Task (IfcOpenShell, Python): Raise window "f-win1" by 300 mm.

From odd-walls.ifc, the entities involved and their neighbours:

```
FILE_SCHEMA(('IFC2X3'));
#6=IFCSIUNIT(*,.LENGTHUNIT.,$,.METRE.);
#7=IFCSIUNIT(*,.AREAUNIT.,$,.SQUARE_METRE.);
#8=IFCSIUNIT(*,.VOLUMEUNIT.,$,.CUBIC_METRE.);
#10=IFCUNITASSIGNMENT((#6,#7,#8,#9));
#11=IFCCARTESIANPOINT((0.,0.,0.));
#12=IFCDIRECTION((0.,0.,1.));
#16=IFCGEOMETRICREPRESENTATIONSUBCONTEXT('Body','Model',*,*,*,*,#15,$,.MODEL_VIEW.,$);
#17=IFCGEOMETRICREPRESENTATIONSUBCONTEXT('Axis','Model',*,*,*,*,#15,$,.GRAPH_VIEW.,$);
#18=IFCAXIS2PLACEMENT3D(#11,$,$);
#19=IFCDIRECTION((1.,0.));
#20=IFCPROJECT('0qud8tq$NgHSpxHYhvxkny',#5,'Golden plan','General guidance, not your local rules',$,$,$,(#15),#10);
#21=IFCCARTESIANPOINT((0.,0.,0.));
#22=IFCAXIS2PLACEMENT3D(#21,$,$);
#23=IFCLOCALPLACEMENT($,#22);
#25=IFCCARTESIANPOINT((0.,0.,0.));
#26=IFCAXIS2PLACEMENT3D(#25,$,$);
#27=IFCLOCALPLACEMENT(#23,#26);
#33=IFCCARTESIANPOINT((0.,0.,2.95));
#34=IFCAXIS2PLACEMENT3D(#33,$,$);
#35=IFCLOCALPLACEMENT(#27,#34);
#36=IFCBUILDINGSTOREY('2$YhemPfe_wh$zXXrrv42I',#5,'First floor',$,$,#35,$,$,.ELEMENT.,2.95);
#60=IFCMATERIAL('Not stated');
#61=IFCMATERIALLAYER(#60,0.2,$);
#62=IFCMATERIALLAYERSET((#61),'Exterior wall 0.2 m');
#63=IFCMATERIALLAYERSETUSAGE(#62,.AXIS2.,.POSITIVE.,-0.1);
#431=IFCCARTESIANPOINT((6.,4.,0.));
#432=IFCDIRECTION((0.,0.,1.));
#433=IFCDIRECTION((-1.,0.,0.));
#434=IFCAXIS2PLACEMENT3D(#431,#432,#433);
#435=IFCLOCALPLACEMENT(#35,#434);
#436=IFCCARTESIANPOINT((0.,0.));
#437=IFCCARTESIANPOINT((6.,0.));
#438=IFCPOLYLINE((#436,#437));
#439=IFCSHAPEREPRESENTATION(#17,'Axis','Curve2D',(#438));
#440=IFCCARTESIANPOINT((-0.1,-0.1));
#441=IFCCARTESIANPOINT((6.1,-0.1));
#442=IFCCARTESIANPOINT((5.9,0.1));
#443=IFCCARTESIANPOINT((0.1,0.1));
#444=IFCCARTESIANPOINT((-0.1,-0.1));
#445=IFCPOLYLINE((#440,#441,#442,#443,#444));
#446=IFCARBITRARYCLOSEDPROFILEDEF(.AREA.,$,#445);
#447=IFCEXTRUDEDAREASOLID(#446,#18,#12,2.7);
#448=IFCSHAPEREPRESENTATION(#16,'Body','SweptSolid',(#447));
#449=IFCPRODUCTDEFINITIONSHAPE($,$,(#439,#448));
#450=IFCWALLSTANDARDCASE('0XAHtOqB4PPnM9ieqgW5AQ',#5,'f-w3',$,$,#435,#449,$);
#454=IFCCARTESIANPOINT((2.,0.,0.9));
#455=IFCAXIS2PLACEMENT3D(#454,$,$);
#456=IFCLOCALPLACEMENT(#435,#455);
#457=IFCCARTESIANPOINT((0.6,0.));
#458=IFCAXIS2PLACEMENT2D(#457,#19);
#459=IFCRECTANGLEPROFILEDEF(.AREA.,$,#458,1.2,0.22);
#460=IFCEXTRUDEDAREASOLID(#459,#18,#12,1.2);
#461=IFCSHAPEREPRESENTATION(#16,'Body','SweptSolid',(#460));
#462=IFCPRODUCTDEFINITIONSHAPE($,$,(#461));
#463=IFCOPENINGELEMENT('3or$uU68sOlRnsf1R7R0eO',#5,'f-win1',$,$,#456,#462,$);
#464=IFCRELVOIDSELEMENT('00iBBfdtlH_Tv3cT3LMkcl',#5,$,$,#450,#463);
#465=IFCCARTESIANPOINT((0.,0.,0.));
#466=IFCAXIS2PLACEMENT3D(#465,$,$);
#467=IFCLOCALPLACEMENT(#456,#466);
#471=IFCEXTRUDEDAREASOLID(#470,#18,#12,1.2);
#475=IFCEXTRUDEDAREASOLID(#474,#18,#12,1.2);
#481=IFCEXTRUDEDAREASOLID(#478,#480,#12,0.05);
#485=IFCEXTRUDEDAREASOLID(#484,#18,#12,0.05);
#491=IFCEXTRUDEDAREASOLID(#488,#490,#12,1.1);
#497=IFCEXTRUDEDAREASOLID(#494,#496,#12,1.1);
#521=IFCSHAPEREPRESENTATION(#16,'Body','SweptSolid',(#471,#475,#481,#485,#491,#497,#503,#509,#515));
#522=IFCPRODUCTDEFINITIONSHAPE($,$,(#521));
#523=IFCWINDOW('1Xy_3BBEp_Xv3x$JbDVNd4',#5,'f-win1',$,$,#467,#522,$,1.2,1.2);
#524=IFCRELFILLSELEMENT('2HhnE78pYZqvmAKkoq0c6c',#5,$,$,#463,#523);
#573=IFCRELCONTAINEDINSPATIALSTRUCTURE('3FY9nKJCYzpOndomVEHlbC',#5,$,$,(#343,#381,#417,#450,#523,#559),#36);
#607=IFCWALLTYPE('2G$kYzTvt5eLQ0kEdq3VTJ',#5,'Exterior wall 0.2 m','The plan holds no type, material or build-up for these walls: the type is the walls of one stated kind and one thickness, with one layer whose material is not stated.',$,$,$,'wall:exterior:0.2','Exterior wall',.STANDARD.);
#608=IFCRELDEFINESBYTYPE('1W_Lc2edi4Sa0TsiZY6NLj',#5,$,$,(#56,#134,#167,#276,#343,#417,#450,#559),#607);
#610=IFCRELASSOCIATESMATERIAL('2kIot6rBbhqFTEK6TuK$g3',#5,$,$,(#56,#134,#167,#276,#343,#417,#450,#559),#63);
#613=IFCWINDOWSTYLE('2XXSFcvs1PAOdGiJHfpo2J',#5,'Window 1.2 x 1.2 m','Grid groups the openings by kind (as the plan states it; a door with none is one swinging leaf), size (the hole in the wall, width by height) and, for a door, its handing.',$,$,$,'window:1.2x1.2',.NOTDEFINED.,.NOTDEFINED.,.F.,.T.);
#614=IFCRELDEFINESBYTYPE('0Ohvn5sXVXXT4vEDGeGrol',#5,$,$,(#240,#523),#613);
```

```python
import numpy as np
import ifcopenshell
import ifcopenshell.api.geometry
import ifcopenshell.util.placement
import ifcopenshell.util.unit

model = ifcopenshell.open("odd-walls.ifc")
unit_scale = ifcopenshell.util.unit.calculate_unit_scale(model)

window = model.by_guid("1Xy_3BBEp_Xv3x$JbDVNd4")
opening = window.FillsVoids[0].RelatingOpeningElement
dz = 0.3

shift = np.array([0.0, 0.0, dz])
# The window is placed relative to its opening, so it follows when the opening moves.
matrix = ifcopenshell.util.placement.get_local_placement(opening.ObjectPlacement)
matrix[:3, 3] += shift
ifcopenshell.api.geometry.edit_object_placement(
    model, product=opening, matrix=matrix, is_si=False, should_transform_children=True
)

print(f"moved by {dz * unit_scale:+.3f} m")

model.write("odd-walls_v2.ifc")
```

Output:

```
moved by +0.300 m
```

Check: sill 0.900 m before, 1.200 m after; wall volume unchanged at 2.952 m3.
